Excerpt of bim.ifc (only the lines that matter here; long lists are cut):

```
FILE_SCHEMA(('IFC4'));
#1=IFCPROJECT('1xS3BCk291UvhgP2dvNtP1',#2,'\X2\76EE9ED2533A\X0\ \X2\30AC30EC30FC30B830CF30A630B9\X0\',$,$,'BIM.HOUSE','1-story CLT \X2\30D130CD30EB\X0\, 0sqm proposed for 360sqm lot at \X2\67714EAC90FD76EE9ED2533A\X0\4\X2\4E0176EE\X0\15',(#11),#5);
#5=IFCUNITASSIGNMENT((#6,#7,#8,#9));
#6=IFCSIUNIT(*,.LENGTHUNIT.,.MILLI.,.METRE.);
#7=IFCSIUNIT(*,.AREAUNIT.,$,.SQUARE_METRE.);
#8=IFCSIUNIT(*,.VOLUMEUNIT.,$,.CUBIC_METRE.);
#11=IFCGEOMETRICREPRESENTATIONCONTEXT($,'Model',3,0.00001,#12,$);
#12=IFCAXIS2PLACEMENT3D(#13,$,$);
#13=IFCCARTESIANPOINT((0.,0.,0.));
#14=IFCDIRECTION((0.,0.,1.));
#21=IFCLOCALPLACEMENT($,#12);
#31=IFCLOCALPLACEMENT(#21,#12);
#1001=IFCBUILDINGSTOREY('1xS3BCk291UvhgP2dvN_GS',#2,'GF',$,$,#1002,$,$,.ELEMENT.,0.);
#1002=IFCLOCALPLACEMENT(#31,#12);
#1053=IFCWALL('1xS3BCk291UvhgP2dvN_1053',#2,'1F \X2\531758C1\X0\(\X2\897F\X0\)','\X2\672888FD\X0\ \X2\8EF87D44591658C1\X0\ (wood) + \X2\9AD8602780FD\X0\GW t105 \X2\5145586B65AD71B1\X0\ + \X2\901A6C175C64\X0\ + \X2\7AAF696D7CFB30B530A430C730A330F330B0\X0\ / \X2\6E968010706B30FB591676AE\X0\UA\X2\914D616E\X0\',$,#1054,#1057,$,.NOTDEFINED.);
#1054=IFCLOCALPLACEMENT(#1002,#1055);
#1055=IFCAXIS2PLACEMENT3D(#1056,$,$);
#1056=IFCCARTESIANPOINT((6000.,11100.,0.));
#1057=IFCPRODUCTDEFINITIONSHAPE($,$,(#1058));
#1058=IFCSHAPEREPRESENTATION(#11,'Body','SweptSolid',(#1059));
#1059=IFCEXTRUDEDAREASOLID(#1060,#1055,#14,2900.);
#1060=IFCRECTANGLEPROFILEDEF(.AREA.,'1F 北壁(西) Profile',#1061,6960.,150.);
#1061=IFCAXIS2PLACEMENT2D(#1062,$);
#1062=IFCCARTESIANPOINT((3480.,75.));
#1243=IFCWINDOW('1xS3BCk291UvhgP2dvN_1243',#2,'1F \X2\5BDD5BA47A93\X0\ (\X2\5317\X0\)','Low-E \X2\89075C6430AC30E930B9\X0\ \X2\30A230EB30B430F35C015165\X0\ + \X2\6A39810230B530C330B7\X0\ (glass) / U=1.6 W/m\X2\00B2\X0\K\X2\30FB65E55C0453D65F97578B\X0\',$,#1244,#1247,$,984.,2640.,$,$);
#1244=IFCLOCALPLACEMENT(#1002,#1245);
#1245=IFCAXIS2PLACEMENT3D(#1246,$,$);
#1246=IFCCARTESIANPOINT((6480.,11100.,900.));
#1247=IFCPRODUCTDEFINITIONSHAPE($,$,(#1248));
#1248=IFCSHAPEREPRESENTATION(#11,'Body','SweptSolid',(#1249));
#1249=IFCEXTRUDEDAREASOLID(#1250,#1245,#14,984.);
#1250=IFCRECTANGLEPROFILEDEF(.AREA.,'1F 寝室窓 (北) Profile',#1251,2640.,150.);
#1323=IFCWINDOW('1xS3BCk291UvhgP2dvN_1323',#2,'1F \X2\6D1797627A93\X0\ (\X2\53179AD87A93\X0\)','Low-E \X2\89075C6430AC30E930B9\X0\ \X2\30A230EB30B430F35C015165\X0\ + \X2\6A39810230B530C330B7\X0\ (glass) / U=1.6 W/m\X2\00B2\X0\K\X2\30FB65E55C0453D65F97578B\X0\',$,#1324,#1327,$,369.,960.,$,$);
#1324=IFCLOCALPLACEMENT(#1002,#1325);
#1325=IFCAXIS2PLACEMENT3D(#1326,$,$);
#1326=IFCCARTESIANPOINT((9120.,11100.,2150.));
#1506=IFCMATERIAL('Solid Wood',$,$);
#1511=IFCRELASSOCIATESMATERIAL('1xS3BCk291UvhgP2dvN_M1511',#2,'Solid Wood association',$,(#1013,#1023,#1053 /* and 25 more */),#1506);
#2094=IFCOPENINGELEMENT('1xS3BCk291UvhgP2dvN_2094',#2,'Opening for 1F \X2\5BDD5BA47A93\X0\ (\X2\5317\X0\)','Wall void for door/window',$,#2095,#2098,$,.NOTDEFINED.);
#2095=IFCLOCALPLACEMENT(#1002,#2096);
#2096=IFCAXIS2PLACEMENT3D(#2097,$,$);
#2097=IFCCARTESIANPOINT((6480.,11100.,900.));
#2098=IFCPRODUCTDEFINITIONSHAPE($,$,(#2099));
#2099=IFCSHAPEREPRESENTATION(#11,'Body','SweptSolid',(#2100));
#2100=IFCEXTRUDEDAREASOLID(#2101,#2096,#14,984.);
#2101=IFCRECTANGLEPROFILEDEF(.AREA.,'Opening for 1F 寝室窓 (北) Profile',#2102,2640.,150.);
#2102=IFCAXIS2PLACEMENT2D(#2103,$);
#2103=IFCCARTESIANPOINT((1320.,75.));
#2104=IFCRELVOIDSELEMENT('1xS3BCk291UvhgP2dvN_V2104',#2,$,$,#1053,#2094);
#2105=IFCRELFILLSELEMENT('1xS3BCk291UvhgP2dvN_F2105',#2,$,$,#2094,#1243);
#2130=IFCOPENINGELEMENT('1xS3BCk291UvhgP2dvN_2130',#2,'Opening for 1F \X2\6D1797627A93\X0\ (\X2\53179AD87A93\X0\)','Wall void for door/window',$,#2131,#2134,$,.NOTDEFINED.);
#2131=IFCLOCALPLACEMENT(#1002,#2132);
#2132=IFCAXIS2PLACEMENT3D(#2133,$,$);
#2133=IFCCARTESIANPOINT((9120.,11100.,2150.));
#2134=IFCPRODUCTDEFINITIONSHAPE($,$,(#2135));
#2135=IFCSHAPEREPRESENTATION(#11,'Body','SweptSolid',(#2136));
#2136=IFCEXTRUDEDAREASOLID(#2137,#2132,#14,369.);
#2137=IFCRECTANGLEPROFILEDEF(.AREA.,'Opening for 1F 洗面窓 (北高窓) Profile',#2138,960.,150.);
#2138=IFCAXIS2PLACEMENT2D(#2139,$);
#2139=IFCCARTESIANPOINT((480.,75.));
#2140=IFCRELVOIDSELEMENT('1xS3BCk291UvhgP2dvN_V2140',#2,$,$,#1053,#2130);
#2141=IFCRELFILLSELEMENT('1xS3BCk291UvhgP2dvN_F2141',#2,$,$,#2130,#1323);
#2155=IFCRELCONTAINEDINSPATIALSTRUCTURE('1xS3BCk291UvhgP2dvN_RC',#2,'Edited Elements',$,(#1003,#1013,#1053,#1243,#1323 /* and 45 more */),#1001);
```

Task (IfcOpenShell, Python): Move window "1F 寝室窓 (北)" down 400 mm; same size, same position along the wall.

```python
import numpy as np
import ifcopenshell
import ifcopenshell.api.geometry
import ifcopenshell.util.placement
import ifcopenshell.util.unit

model = ifcopenshell.open("bim.ifc")
unit_scale = ifcopenshell.util.unit.calculate_unit_scale(model)

window = model.by_id(1243)
opening = window.FillsVoids[0].RelatingOpeningElement
dz = -0.4 / unit_scale

shift = np.array([0.0, 0.0, dz])
# The window is not placed relative to its opening, so move both.
for product in (opening, window):
    matrix = ifcopenshell.util.placement.get_local_placement(product.ObjectPlacement)
    matrix[:3, 3] += shift
    ifcopenshell.api.geometry.edit_object_placement(model, product=product, matrix=matrix, is_si=False)

print(f"moved by {dz * unit_scale:+.3f} m")

model.write("bim_v2.ifc")
```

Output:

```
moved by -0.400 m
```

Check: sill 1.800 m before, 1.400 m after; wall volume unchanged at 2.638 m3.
